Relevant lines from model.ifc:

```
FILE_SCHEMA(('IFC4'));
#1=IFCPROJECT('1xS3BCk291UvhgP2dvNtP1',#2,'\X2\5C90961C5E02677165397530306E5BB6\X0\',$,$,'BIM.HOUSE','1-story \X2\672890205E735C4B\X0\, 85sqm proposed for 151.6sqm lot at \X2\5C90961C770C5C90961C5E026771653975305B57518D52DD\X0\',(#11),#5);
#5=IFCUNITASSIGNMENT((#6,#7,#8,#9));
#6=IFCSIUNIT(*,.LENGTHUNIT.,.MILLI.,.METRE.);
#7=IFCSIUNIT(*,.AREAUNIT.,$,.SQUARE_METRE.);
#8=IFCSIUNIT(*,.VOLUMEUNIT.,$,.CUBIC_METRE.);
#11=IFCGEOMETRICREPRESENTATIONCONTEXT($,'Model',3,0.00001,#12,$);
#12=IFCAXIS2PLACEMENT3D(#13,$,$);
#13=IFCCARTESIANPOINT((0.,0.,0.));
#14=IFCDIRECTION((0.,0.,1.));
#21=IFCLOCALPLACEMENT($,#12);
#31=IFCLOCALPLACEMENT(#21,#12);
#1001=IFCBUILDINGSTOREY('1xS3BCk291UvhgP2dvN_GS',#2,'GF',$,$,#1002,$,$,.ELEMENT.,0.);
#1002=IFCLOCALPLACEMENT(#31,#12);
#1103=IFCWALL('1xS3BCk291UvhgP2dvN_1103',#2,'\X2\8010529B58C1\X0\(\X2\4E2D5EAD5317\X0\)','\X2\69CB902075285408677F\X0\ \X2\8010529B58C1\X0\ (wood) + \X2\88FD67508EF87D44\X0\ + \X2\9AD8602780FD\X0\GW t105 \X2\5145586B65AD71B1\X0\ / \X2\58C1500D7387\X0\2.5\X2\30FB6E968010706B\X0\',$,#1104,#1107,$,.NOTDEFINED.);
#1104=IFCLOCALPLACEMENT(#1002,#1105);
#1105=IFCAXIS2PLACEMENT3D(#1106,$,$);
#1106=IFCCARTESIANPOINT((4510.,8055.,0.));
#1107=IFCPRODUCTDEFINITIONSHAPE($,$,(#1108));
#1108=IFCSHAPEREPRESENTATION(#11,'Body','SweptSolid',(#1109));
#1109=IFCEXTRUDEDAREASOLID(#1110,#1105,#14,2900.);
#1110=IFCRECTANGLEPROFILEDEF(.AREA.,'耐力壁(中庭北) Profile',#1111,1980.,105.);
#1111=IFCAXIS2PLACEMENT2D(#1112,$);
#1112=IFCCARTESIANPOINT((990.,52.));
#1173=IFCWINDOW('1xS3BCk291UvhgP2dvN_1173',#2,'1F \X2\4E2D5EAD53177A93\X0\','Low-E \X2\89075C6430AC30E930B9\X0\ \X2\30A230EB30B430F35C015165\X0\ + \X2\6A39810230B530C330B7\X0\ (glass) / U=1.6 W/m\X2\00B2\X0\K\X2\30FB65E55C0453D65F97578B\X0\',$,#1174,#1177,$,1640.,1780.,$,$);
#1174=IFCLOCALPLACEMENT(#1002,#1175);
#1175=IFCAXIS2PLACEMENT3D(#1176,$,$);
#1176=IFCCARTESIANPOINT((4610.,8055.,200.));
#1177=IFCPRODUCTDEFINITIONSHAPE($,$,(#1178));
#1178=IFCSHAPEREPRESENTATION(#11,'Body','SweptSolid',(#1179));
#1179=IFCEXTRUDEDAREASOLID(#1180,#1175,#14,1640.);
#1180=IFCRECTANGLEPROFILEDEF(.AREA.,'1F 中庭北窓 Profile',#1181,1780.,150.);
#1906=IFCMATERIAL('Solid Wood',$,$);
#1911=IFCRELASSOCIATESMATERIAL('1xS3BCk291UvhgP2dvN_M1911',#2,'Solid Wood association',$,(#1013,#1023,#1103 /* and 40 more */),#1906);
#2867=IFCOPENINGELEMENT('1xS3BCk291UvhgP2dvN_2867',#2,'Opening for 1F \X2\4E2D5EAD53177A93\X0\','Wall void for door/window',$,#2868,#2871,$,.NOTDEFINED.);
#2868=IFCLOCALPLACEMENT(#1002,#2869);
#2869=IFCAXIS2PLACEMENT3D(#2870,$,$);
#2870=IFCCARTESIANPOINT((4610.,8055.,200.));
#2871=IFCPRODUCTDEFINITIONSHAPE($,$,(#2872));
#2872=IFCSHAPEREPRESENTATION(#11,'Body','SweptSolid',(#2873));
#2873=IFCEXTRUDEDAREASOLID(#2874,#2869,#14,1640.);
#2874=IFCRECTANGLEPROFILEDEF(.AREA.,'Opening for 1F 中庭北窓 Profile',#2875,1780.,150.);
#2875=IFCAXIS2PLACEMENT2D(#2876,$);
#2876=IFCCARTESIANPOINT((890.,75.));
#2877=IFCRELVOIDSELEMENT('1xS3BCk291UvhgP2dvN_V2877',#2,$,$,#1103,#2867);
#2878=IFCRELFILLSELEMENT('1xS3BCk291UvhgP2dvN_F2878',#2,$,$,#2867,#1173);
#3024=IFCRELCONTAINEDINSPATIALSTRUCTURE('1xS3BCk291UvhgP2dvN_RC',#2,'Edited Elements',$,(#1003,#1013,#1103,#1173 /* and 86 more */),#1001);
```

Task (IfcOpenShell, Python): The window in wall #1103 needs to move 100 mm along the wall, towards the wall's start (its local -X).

```python
import ifcopenshell
import ifcopenshell.api.geometry
import ifcopenshell.util.placement

model = ifcopenshell.open("model.ifc")

window = model.by_guid("1xS3BCk291UvhgP2dvN_1173")
opening = window.FillsVoids[0].RelatingOpeningElement
wall = opening.VoidsElements[0].RelatingBuildingElement

wall_matrix = ifcopenshell.util.placement.get_local_placement(wall.ObjectPlacement)
shift = wall_matrix[:3, 0] * -100.0
before = ifcopenshell.util.placement.get_local_placement(window.ObjectPlacement)[:3, 3].copy()

# The window is not placed relative to its opening, so move both.
for product in (opening, window):
    matrix = ifcopenshell.util.placement.get_local_placement(product.ObjectPlacement)
    matrix[:3, 3] += shift
    ifcopenshell.api.geometry.edit_object_placement(model, product=product, matrix=matrix, is_si=False)

after = ifcopenshell.util.placement.get_local_placement(window.ObjectPlacement)[:3, 3]
print("window moved by", (after - before).round(3) + 0.0)

model.write("model-out.ifc")
```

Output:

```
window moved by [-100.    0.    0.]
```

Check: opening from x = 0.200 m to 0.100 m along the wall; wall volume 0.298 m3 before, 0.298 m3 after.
